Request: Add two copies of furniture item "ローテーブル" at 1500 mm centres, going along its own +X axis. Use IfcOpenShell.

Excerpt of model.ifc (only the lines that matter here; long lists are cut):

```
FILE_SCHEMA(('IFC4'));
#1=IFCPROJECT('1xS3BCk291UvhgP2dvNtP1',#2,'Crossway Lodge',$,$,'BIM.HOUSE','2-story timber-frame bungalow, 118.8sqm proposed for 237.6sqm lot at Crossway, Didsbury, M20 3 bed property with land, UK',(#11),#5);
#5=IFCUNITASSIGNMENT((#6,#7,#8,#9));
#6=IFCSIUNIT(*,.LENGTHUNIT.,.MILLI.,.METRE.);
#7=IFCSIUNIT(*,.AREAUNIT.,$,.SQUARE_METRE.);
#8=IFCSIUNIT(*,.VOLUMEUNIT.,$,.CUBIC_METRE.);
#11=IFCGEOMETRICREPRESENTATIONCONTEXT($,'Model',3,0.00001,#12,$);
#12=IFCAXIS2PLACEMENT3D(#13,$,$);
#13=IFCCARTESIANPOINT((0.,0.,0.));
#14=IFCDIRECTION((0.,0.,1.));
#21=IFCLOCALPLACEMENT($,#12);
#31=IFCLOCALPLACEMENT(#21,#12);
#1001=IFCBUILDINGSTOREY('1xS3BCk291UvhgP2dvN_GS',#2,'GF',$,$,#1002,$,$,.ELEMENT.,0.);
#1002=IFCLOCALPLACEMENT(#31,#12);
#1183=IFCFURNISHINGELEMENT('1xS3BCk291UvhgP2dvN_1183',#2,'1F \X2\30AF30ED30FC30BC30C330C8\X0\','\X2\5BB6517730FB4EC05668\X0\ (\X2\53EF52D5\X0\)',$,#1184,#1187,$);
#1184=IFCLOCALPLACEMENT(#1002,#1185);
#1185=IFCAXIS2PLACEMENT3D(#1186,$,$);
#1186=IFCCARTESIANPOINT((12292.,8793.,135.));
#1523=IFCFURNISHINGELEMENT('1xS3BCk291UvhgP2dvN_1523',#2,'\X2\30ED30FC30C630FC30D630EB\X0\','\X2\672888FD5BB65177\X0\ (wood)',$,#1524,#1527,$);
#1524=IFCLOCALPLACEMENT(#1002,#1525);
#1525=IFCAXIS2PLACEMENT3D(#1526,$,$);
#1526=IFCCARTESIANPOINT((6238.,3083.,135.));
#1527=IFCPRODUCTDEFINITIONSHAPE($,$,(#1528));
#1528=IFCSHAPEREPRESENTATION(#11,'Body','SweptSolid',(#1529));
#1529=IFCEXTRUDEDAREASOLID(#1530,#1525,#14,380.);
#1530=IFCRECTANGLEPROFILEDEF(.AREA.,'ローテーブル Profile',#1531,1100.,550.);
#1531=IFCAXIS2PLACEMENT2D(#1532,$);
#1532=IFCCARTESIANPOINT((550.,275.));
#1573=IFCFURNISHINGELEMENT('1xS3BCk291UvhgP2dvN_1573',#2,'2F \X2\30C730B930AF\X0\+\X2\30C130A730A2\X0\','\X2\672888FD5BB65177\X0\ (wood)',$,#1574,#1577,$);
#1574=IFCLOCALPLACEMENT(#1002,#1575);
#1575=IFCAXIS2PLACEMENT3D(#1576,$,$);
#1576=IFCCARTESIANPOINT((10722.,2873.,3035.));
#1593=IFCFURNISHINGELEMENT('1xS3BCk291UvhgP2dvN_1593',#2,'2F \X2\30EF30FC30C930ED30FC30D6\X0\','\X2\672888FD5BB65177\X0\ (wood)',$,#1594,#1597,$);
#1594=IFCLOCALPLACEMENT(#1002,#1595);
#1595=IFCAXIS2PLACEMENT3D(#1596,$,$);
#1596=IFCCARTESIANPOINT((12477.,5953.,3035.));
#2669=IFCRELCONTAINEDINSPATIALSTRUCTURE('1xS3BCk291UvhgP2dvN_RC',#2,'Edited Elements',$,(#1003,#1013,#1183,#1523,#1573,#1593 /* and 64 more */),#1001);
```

```python
import ifcopenshell
import ifcopenshell.api.geometry
import ifcopenshell.api.root
import ifcopenshell.util.element
import ifcopenshell.util.placement

model = ifcopenshell.open("model.ifc")


def reuse_history(source, copy):
    """copy_class also copies each property set's owner history, people and application; keep the originals."""
    for rel in copy.IsDefinedBy:
        if rel.is_a("IfcRelDefinesByProperties") and (history := rel.RelatingPropertyDefinition.OwnerHistory):
            rel.RelatingPropertyDefinition.OwnerHistory = source.OwnerHistory
            ifcopenshell.util.element.remove_deep2(model, history)


source = model.by_guid("1xS3BCk291UvhgP2dvN_1523")
base = ifcopenshell.util.placement.get_local_placement(source.ObjectPlacement)
step = base[:3, 0] * 1500.0

for i in range(1, 3):
    copy = ifcopenshell.api.root.copy_class(model, product=source)
    copy.Representation = ifcopenshell.util.element.copy_deep(
        model, source.Representation, exclude=["IfcGeometricRepresentationContext", "IfcRepresentationMap"]
    )
    reuse_history(source, copy)
    matrix = base.copy()
    matrix[:3, 3] += i * step
    print("added at", matrix[:3, 3].round(3) + 0.0)
    ifcopenshell.api.geometry.edit_object_placement(model, product=copy, matrix=matrix, is_si=False)

model.write("model_rev.ifc")
```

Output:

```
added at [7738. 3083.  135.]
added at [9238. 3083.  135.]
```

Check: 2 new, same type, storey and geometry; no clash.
